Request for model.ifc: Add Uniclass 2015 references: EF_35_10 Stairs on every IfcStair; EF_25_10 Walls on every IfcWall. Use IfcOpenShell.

First a look at what the model holds.

```python
import ifcopenshell

model = ifcopenshell.open("model.ifc")
print(model.schema)
print("classifications:", [c.Name for c in model.by_type("IfcClassification")])
for ifc_class in ("IfcDoor", "IfcRoof", "IfcStair", "IfcWall", "IfcWindow"):
    print(ifc_class, len(model.by_type(ifc_class)))
```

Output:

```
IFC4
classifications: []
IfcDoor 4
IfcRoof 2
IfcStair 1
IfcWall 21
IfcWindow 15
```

```python
import ifcopenshell
import ifcopenshell.api.classification

model = ifcopenshell.open("model.ifc")

system = ifcopenshell.api.classification.add_classification(model, classification="Uniclass 2015")

codes = {
    "IfcStair": ("EF_35_10", "Stairs"),
    "IfcWall": ("EF_25_10", "Walls"),
}
for ifc_class, (code, name) in codes.items():
    products = model.by_type(ifc_class)
    ifcopenshell.api.classification.add_reference(
        model, products=products, classification=system, identification=code, name=name
    )
    print(code, len(products))

model.write("model_v2.ifc")
```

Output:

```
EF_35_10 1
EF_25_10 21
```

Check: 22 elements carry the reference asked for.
